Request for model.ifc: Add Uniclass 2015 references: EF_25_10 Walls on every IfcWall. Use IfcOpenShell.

First a look at what the model holds.

```python
import ifcopenshell

model = ifcopenshell.open("model.ifc")
print(model.schema)
print("classifications:", [c.Name for c in model.by_type("IfcClassification")])
for ifc_class in ("IfcDoor", "IfcRoof", "IfcStair", "IfcWall", "IfcWindow"):
    print(ifc_class, len(model.by_type(ifc_class)))
```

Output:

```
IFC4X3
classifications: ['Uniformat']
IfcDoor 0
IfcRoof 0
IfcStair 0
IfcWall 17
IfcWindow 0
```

```python
import ifcopenshell
import ifcopenshell.api.classification

model = ifcopenshell.open("model.ifc")

system = ifcopenshell.api.classification.add_classification(model, classification="Uniclass 2015")

codes = {
    "IfcWall": ("EF_25_10", "Walls"),
}
for ifc_class, (code, name) in codes.items():
    products = model.by_type(ifc_class)
    ifcopenshell.api.classification.add_reference(
        model, products=products, classification=system, identification=code, name=name
    )
    print(code, len(products))

model.write("model_rev.ifc")
```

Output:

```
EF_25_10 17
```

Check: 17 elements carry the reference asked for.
